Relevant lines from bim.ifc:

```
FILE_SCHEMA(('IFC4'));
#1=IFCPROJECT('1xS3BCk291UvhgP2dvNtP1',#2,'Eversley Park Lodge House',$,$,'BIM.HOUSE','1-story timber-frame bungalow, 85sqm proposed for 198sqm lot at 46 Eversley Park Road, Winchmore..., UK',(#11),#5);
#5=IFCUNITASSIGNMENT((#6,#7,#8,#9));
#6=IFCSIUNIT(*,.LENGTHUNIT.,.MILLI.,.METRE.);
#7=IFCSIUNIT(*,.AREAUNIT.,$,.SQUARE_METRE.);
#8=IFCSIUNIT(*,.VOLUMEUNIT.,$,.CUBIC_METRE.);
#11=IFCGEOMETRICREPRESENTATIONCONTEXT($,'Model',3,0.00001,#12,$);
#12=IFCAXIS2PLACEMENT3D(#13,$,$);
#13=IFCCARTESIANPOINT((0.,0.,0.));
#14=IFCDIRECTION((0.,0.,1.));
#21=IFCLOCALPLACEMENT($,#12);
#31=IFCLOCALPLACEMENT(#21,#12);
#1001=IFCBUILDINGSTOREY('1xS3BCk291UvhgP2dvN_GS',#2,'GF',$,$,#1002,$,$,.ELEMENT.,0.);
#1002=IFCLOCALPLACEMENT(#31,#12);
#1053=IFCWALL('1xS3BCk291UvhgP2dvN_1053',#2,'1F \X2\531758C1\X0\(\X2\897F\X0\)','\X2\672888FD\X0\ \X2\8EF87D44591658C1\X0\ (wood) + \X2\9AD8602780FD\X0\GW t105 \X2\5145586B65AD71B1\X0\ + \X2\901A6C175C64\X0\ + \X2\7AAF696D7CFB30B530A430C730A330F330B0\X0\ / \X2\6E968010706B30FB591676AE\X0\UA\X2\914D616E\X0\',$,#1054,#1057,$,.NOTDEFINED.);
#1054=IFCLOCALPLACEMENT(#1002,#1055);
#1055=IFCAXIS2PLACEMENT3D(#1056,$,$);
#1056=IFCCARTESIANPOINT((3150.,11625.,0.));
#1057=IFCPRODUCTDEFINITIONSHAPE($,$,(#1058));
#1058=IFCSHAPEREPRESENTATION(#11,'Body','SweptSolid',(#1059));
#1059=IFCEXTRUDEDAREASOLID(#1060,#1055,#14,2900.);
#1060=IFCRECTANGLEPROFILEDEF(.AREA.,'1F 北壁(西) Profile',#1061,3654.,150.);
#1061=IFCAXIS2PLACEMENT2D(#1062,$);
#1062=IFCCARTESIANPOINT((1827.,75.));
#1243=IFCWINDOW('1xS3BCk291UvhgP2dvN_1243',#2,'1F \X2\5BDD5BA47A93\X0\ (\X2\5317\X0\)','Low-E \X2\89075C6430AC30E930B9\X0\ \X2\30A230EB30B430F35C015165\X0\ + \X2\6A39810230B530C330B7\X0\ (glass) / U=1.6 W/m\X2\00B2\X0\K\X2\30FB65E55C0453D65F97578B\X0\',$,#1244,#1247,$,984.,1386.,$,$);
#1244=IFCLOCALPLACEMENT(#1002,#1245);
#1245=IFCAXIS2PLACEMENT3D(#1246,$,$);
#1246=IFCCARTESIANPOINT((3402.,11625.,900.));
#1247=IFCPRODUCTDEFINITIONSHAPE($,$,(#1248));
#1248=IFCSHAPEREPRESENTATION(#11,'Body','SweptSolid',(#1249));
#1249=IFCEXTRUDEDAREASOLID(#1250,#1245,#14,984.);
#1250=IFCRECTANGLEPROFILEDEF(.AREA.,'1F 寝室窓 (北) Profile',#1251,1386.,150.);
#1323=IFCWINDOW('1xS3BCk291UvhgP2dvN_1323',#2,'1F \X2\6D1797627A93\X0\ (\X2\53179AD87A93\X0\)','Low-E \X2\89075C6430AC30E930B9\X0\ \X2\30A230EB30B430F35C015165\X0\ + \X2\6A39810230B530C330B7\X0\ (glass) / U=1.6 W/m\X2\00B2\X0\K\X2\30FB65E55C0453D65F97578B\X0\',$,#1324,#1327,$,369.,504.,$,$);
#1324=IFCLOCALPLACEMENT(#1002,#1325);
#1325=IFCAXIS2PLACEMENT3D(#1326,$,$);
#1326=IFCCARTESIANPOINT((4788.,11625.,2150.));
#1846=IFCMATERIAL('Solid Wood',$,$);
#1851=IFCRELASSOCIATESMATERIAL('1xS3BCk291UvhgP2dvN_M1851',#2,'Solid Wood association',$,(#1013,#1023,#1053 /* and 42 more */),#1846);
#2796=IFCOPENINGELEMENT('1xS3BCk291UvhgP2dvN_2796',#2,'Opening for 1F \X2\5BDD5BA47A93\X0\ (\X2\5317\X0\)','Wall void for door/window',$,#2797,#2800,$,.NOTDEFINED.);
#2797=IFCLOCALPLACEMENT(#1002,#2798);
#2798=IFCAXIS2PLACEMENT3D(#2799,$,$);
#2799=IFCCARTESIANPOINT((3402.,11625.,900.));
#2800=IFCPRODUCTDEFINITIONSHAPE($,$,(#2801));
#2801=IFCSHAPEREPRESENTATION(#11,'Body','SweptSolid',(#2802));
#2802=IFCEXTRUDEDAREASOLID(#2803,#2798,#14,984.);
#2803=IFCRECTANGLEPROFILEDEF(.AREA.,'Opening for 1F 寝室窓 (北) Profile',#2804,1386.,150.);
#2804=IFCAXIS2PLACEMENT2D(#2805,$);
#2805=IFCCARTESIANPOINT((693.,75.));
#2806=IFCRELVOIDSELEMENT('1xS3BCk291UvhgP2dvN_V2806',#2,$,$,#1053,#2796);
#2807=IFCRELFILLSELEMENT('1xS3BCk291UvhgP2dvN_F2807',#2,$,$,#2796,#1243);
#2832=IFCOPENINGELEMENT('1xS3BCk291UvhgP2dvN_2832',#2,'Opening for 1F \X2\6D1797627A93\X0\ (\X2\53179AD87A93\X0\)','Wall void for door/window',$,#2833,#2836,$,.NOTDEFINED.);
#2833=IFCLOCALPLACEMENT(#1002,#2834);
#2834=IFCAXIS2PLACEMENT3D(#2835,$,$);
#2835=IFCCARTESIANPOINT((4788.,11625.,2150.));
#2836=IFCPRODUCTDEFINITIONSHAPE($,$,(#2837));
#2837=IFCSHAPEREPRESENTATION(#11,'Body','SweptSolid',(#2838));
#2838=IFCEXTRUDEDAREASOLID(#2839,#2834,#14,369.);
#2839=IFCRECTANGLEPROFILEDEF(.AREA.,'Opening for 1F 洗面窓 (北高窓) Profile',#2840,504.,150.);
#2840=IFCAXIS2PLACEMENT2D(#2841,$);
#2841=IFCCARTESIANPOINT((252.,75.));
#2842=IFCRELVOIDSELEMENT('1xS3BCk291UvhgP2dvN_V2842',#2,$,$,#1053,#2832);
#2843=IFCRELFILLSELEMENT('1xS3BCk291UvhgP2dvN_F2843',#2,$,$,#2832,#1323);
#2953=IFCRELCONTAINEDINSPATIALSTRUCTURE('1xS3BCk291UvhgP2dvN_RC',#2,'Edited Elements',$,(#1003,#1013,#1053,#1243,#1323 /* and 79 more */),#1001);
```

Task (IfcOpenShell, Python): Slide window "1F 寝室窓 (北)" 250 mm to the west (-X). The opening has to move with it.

```python
import ifcopenshell
import ifcopenshell.api.geometry
import ifcopenshell.util.placement
import ifcopenshell.util.unit

model = ifcopenshell.open("bim.ifc")
unit_scale = ifcopenshell.util.unit.calculate_unit_scale(model)

window = model.by_id(1243)
opening = window.FillsVoids[0].RelatingOpeningElement
wall = opening.VoidsElements[0].RelatingBuildingElement

wall_matrix = ifcopenshell.util.placement.get_local_placement(wall.ObjectPlacement)
shift = wall_matrix[:3, 0] * -0.25 / unit_scale
before = ifcopenshell.util.placement.get_local_placement(window.ObjectPlacement)[:3, 3].copy()

# The window is not placed relative to its opening, so move both.
for product in (opening, window):
    matrix = ifcopenshell.util.placement.get_local_placement(product.ObjectPlacement)
    matrix[:3, 3] += shift
    ifcopenshell.api.geometry.edit_object_placement(model, product=product, matrix=matrix, is_si=False)

after = ifcopenshell.util.placement.get_local_placement(window.ObjectPlacement)[:3, 3]
print("window moved by", (after - before).round(3) + 0.0)

model.write("bim_rev.ifc")
```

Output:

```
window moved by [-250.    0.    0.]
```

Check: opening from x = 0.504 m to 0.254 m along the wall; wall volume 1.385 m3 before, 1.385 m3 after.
